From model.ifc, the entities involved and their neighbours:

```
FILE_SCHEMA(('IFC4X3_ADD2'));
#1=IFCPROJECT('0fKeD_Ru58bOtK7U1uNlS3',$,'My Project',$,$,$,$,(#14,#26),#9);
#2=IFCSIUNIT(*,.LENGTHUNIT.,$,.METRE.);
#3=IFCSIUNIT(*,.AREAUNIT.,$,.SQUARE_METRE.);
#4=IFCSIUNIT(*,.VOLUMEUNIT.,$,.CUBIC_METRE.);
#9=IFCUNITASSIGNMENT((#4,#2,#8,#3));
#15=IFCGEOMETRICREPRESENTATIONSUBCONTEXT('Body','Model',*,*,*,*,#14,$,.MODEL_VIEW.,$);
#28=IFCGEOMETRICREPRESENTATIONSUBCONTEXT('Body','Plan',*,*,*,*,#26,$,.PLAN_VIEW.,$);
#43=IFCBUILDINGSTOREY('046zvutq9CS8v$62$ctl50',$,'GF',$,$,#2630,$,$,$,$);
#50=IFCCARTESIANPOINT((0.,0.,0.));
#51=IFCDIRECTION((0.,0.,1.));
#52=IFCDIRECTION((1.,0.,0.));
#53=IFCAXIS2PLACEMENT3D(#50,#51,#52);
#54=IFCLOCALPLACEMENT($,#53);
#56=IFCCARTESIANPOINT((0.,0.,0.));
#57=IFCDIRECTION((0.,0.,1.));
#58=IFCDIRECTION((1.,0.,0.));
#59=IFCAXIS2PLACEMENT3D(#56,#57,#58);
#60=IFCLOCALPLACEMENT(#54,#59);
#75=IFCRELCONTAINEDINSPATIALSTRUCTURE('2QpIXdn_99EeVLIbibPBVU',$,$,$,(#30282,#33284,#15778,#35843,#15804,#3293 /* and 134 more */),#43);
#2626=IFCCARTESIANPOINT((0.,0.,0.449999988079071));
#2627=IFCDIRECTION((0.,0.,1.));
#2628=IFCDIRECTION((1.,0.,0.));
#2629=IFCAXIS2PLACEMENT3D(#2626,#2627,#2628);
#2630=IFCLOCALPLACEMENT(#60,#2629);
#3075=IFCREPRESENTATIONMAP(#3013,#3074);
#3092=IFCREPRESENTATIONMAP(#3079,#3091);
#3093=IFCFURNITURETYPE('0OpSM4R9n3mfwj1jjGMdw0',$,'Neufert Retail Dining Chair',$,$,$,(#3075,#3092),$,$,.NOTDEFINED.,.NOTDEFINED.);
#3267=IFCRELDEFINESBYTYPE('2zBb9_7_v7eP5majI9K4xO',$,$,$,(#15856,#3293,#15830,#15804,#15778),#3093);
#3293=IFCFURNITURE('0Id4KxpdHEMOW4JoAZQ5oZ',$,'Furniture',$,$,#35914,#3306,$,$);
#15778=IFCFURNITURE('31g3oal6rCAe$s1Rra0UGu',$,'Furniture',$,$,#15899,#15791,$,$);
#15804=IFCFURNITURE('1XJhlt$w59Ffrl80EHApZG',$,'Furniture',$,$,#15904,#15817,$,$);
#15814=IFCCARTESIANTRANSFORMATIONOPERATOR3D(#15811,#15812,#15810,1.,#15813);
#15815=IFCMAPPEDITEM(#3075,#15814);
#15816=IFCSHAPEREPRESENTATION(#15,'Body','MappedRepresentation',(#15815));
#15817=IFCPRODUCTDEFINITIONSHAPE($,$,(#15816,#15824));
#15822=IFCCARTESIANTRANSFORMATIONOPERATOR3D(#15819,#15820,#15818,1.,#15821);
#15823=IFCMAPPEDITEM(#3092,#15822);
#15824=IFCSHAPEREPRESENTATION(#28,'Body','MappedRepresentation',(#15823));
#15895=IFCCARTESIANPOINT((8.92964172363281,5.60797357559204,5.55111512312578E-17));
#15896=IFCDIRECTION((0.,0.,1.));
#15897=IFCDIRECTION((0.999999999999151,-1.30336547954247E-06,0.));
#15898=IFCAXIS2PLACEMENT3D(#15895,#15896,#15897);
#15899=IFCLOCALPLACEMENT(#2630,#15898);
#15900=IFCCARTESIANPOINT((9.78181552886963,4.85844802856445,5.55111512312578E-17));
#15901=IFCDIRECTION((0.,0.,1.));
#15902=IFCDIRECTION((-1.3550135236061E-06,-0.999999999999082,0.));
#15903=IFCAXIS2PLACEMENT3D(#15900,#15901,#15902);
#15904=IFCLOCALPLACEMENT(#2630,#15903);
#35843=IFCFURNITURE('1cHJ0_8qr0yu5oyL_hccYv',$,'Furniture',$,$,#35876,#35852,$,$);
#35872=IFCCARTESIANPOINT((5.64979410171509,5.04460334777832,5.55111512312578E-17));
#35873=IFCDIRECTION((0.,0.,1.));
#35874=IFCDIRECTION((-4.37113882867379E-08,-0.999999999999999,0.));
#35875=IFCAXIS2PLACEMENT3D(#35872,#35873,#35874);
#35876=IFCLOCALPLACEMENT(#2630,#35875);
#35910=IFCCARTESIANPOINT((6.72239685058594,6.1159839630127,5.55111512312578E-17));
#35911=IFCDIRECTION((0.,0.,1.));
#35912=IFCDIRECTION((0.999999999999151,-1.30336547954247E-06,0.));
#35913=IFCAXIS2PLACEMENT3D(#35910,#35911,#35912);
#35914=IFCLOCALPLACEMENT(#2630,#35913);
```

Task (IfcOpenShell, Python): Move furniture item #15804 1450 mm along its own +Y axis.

```python
import ifcopenshell
import ifcopenshell.api.geometry
import ifcopenshell.util.placement

model = ifcopenshell.open("model.ifc")

item = model.by_id(15804)
matrix = ifcopenshell.util.placement.get_local_placement(item.ObjectPlacement)
matrix[:3, 3] += matrix[:3, 1] * 1.45
ifcopenshell.api.geometry.edit_object_placement(model, product=item, matrix=matrix, is_si=False)

print(ifcopenshell.util.placement.get_local_placement(item.ObjectPlacement).round(3) + 0.0)

model.write("model_v2.ifc")
```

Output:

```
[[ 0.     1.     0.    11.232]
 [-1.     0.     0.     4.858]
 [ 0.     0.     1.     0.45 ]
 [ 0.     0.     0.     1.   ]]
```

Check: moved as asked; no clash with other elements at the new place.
